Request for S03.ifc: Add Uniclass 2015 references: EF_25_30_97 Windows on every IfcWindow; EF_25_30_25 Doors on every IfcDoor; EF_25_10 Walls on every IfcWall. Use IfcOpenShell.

First a look at what the model holds.

```python
import ifcopenshell

model = ifcopenshell.open("S03.ifc")
print(model.schema)
print("classifications:", [c.Name for c in model.by_type("IfcClassification")])
for ifc_class in ("IfcDoor", "IfcRoof", "IfcStair", "IfcWall", "IfcWindow"):
    print(ifc_class, len(model.by_type(ifc_class)))
```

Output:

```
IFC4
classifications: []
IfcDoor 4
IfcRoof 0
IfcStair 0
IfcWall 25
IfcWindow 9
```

```python
import ifcopenshell
import ifcopenshell.api.classification

model = ifcopenshell.open("S03.ifc")

system = ifcopenshell.api.classification.add_classification(model, classification="Uniclass 2015")

codes = {
    "IfcWindow": ("EF_25_30_97", "Windows"),
    "IfcDoor": ("EF_25_30_25", "Doors"),
    "IfcWall": ("EF_25_10", "Walls"),
}
for ifc_class, (code, name) in codes.items():
    products = model.by_type(ifc_class)
    ifcopenshell.api.classification.add_reference(
        model, products=products, classification=system, identification=code, name=name
    )
    print(code, len(products))

model.write("S03-out.ifc")
```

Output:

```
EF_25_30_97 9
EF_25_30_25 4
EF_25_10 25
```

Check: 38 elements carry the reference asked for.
